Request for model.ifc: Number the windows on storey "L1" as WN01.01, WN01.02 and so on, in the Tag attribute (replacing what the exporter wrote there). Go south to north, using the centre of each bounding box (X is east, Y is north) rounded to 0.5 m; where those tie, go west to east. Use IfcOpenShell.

First a look at what the model holds.

```python
import ifcopenshell
import ifcopenshell.util.element
import ifcopenshell.util.placement

model = ifcopenshell.open("model.ifc")
print(model.schema)
storey = next(s for s in model.by_type("IfcBuildingStorey") if s.Name == "L1")
windows = [e for e in ifcopenshell.util.element.get_decomposition(storey) if e.is_a("IfcWindow")]
for e in sorted(windows, key=lambda e: e.id()):
    origin = ifcopenshell.util.placement.get_local_placement(e.ObjectPlacement)[:3, 3]
    print(e.id(), e.Tag, e.Name, origin.round(2) + 0.0, sep=" | ")
```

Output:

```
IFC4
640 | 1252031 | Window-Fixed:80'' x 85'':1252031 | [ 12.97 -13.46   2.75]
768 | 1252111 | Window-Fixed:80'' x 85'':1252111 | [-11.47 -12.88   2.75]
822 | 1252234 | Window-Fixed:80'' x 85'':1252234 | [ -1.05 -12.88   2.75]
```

```python
import ifcopenshell
import ifcopenshell.geom
import ifcopenshell.util.element
import ifcopenshell.util.shape

model = ifcopenshell.open("model.ifc")
settings = ifcopenshell.geom.settings()
settings.set("use-world-coords", True)


def centre(element):
    shape = ifcopenshell.geom.create_shape(settings, element)
    return ifcopenshell.util.shape.get_bbox_centroid(shape.geometry)


storey = next(s for s in model.by_type("IfcBuildingStorey") if s.Name == "L1")
windows = [e for e in ifcopenshell.util.element.get_decomposition(storey) if e.is_a("IfcWindow")]

# Insertion points can sit at a corner or the storey origin, so sort by the geometry (in metres).
centres = {e: centre(e) for e in windows}
windows.sort(key=lambda e: (round(centres[e][1] / 0.5), centres[e][0]))

for i, e in enumerate(windows, start=1):
    number = f"WN01.{i:02d}"
    e.Tag = number
    print(e.id(), number)

model.write("model-out.ifc")
```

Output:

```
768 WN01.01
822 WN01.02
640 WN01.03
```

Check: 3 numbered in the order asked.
